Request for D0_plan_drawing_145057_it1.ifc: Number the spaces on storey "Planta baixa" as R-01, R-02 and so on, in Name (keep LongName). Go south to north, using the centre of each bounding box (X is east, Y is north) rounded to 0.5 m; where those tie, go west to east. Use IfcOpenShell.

First a look at what the model holds.

```python
import ifcopenshell
import ifcopenshell.util.element
import ifcopenshell.util.placement

model = ifcopenshell.open("D0_plan_drawing_145057_it1.ifc")
print(model.schema)
storey = next(s for s in model.by_type("IfcBuildingStorey") if s.Name == "Planta baixa")
spaces = [e for e in ifcopenshell.util.element.get_decomposition(storey) if e.is_a("IfcSpace")]
for e in sorted(spaces, key=lambda e: e.id()):
    origin = ifcopenshell.util.placement.get_local_placement(e.ObjectPlacement)[:3, 3]
    print(e.id(), e.Name, e.LongName, origin.round(2) + 0.0, sep=" | ")
```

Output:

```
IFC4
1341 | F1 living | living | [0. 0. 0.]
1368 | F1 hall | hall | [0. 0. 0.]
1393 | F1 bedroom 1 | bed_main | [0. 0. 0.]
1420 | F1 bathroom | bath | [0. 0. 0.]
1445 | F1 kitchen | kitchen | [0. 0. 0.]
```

```python
import ifcopenshell
import ifcopenshell.geom
import ifcopenshell.util.element
import ifcopenshell.util.shape

model = ifcopenshell.open("D0_plan_drawing_145057_it1.ifc")
settings = ifcopenshell.geom.settings()
settings.set("use-world-coords", True)


def centre(element):
    shape = ifcopenshell.geom.create_shape(settings, element)
    return ifcopenshell.util.shape.get_bbox_centroid(shape.geometry)


storey = next(s for s in model.by_type("IfcBuildingStorey") if s.Name == "Planta baixa")
spaces = [e for e in ifcopenshell.util.element.get_decomposition(storey) if e.is_a("IfcSpace")]

# Insertion points can sit at a corner or the storey origin, so sort by the geometry (in metres).
centres = {e: centre(e) for e in spaces}
spaces.sort(key=lambda e: (round(centres[e][1] / 0.5), centres[e][0]))

for i, e in enumerate(spaces, start=1):
    number = f"R-{i:02d}"
    e.Name = number
    print(e.id(), number)

model.write("D0_plan_drawing_145057_it1-out.ifc")
```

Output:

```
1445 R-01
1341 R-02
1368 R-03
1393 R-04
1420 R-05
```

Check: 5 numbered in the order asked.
